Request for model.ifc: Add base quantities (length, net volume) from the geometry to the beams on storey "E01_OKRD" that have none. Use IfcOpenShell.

First a look at what the model holds.

```python
import ifcopenshell
import ifcopenshell.util.element
import ifcopenshell.util.unit

model = ifcopenshell.open("model.ifc")
print(model.schema)
for unit_type in ("LENGTHUNIT", "AREAUNIT", "VOLUMEUNIT"):
    print(unit_type, ifcopenshell.util.unit.calculate_unit_scale(model, unit_type))
storey = next(s for s in model.by_type("IfcBuildingStorey") if s.Name == "E01_OKRD")
beams = [e for e in ifcopenshell.util.element.get_decomposition(storey) if e.is_a("IfcBeam")]
for e in sorted(beams, key=lambda e: e.id()):
    print(e.id(), e.is_a(), e.Name, list(ifcopenshell.util.element.get_psets(e, qtos_only=True)), sep=" | ")
```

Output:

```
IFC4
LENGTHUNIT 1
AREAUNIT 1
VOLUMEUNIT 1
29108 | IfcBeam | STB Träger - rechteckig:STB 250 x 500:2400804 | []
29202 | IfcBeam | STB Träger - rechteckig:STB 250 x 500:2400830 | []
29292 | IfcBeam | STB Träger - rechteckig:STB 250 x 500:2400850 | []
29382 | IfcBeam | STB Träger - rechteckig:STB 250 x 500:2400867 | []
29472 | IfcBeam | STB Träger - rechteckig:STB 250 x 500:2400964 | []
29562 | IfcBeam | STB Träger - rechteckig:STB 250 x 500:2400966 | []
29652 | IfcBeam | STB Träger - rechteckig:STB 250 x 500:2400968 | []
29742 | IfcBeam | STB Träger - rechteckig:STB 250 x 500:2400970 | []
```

```python
import ifcopenshell
import ifcopenshell.api.pset
import ifcopenshell.geom
import ifcopenshell.util.element
import ifcopenshell.util.shape
import ifcopenshell.util.unit

model = ifcopenshell.open("model.ifc")
unit_scale = ifcopenshell.util.unit.calculate_unit_scale(model)
volume_scale = ifcopenshell.util.unit.calculate_unit_scale(model, "VOLUMEUNIT")
settings = ifcopenshell.geom.settings()

storey = next(s for s in model.by_type("IfcBuildingStorey") if s.Name == "E01_OKRD")
beams = [e for e in ifcopenshell.util.element.get_decomposition(storey) if e.is_a("IfcBeam")]

for e in sorted(beams, key=lambda e: e.id()):
    if ifcopenshell.util.element.get_psets(e, qtos_only=True, should_inherit=False):
        continue
    # Geometry comes back in metres, in the element's own axes.
    shape = ifcopenshell.geom.create_shape(settings, e)
    values = {
        "Length": ifcopenshell.util.shape.get_max_xyz(shape.geometry) / unit_scale,
        "NetVolume": ifcopenshell.util.shape.get_volume(shape.geometry) / volume_scale,
    }
    qto = ifcopenshell.api.pset.add_qto(model, product=e, name="Qto_BeamBaseQuantities")
    ifcopenshell.api.pset.edit_qto(model, qto=qto, properties=values)
    print(e.id(), {k: round(v, 3) for k, v in values.items()})

model.write("model_edited.ifc")
```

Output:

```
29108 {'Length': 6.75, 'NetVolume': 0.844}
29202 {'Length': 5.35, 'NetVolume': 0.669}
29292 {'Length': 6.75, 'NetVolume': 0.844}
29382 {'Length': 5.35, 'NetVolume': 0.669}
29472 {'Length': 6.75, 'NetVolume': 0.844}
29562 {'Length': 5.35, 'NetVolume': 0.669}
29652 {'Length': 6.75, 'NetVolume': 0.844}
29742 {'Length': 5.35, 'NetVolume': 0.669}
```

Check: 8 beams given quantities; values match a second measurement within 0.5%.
